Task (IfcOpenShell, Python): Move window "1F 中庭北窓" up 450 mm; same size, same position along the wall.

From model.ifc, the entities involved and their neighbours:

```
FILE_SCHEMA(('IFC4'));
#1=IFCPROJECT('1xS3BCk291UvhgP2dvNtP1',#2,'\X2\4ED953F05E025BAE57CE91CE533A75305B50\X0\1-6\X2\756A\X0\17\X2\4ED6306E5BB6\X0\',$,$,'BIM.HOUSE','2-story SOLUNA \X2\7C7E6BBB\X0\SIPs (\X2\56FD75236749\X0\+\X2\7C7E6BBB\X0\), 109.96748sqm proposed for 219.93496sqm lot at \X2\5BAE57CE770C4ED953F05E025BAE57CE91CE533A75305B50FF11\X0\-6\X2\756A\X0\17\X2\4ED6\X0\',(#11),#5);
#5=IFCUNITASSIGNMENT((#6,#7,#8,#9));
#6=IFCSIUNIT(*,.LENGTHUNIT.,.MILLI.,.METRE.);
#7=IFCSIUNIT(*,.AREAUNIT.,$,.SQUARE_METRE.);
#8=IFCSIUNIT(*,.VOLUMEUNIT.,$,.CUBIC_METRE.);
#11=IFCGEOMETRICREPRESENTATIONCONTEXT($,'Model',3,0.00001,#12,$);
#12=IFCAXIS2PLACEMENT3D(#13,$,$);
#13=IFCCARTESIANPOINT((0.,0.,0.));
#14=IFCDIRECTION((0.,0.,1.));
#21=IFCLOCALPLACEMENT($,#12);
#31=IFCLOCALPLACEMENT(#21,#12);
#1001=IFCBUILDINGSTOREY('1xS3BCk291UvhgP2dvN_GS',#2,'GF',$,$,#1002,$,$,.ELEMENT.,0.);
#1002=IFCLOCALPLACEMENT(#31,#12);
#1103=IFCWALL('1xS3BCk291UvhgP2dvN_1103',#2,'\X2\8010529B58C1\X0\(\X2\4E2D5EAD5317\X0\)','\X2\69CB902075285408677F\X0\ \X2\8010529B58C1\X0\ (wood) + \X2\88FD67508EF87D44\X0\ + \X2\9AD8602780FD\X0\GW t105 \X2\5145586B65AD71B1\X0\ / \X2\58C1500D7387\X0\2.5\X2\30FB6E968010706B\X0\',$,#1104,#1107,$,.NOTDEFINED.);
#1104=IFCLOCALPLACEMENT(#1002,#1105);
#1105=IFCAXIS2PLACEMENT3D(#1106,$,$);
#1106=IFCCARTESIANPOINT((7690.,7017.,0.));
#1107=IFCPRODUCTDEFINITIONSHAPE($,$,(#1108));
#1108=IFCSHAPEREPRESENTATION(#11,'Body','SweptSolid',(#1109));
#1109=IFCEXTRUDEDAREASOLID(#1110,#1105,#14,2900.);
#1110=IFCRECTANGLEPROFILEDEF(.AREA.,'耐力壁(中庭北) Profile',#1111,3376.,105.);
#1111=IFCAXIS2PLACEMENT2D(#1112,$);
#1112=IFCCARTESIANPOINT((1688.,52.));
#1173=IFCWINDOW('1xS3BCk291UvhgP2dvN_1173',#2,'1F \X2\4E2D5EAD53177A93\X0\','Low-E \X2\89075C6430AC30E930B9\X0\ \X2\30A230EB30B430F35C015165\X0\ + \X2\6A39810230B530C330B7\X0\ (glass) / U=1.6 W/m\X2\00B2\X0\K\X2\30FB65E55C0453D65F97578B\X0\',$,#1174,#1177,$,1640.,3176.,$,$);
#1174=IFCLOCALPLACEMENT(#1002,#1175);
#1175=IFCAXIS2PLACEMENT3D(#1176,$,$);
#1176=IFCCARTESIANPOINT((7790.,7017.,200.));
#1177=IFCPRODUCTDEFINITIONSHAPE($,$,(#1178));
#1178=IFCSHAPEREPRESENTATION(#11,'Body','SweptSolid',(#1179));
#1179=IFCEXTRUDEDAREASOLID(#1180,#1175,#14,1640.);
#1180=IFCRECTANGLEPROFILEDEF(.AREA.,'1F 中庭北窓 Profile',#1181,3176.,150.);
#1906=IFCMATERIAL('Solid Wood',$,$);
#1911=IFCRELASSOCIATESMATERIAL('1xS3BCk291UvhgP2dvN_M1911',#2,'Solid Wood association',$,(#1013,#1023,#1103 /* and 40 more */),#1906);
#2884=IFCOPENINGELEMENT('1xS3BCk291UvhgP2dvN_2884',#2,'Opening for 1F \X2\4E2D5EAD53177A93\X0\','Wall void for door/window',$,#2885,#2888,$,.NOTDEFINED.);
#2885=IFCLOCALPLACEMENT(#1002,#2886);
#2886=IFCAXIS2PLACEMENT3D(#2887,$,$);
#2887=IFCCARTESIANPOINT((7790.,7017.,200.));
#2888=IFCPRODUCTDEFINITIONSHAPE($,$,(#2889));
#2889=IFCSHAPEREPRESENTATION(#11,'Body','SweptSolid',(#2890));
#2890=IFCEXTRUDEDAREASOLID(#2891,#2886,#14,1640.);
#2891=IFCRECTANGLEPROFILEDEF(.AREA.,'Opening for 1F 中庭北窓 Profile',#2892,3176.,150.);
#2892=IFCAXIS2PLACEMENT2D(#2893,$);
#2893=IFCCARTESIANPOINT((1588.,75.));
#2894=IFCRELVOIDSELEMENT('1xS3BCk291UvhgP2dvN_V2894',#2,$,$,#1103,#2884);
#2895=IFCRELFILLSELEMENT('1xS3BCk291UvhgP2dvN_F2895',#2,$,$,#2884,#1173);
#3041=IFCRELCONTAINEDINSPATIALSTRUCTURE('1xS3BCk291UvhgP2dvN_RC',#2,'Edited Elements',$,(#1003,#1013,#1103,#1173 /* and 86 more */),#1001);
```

```python
import numpy as np
import ifcopenshell
import ifcopenshell.api.geometry
import ifcopenshell.util.placement
import ifcopenshell.util.unit

model = ifcopenshell.open("model.ifc")
unit_scale = ifcopenshell.util.unit.calculate_unit_scale(model)

window = model.by_id(1173)
opening = window.FillsVoids[0].RelatingOpeningElement
dz = 450.0

shift = np.array([0.0, 0.0, dz])
# The window is not placed relative to its opening, so move both.
for product in (opening, window):
    matrix = ifcopenshell.util.placement.get_local_placement(product.ObjectPlacement)
    matrix[:3, 3] += shift
    ifcopenshell.api.geometry.edit_object_placement(model, product=product, matrix=matrix, is_si=False)

print(f"moved by {dz * unit_scale:+.3f} m")

model.write("model_updated.ifc")
```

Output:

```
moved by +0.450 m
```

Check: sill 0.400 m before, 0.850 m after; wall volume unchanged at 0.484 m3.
